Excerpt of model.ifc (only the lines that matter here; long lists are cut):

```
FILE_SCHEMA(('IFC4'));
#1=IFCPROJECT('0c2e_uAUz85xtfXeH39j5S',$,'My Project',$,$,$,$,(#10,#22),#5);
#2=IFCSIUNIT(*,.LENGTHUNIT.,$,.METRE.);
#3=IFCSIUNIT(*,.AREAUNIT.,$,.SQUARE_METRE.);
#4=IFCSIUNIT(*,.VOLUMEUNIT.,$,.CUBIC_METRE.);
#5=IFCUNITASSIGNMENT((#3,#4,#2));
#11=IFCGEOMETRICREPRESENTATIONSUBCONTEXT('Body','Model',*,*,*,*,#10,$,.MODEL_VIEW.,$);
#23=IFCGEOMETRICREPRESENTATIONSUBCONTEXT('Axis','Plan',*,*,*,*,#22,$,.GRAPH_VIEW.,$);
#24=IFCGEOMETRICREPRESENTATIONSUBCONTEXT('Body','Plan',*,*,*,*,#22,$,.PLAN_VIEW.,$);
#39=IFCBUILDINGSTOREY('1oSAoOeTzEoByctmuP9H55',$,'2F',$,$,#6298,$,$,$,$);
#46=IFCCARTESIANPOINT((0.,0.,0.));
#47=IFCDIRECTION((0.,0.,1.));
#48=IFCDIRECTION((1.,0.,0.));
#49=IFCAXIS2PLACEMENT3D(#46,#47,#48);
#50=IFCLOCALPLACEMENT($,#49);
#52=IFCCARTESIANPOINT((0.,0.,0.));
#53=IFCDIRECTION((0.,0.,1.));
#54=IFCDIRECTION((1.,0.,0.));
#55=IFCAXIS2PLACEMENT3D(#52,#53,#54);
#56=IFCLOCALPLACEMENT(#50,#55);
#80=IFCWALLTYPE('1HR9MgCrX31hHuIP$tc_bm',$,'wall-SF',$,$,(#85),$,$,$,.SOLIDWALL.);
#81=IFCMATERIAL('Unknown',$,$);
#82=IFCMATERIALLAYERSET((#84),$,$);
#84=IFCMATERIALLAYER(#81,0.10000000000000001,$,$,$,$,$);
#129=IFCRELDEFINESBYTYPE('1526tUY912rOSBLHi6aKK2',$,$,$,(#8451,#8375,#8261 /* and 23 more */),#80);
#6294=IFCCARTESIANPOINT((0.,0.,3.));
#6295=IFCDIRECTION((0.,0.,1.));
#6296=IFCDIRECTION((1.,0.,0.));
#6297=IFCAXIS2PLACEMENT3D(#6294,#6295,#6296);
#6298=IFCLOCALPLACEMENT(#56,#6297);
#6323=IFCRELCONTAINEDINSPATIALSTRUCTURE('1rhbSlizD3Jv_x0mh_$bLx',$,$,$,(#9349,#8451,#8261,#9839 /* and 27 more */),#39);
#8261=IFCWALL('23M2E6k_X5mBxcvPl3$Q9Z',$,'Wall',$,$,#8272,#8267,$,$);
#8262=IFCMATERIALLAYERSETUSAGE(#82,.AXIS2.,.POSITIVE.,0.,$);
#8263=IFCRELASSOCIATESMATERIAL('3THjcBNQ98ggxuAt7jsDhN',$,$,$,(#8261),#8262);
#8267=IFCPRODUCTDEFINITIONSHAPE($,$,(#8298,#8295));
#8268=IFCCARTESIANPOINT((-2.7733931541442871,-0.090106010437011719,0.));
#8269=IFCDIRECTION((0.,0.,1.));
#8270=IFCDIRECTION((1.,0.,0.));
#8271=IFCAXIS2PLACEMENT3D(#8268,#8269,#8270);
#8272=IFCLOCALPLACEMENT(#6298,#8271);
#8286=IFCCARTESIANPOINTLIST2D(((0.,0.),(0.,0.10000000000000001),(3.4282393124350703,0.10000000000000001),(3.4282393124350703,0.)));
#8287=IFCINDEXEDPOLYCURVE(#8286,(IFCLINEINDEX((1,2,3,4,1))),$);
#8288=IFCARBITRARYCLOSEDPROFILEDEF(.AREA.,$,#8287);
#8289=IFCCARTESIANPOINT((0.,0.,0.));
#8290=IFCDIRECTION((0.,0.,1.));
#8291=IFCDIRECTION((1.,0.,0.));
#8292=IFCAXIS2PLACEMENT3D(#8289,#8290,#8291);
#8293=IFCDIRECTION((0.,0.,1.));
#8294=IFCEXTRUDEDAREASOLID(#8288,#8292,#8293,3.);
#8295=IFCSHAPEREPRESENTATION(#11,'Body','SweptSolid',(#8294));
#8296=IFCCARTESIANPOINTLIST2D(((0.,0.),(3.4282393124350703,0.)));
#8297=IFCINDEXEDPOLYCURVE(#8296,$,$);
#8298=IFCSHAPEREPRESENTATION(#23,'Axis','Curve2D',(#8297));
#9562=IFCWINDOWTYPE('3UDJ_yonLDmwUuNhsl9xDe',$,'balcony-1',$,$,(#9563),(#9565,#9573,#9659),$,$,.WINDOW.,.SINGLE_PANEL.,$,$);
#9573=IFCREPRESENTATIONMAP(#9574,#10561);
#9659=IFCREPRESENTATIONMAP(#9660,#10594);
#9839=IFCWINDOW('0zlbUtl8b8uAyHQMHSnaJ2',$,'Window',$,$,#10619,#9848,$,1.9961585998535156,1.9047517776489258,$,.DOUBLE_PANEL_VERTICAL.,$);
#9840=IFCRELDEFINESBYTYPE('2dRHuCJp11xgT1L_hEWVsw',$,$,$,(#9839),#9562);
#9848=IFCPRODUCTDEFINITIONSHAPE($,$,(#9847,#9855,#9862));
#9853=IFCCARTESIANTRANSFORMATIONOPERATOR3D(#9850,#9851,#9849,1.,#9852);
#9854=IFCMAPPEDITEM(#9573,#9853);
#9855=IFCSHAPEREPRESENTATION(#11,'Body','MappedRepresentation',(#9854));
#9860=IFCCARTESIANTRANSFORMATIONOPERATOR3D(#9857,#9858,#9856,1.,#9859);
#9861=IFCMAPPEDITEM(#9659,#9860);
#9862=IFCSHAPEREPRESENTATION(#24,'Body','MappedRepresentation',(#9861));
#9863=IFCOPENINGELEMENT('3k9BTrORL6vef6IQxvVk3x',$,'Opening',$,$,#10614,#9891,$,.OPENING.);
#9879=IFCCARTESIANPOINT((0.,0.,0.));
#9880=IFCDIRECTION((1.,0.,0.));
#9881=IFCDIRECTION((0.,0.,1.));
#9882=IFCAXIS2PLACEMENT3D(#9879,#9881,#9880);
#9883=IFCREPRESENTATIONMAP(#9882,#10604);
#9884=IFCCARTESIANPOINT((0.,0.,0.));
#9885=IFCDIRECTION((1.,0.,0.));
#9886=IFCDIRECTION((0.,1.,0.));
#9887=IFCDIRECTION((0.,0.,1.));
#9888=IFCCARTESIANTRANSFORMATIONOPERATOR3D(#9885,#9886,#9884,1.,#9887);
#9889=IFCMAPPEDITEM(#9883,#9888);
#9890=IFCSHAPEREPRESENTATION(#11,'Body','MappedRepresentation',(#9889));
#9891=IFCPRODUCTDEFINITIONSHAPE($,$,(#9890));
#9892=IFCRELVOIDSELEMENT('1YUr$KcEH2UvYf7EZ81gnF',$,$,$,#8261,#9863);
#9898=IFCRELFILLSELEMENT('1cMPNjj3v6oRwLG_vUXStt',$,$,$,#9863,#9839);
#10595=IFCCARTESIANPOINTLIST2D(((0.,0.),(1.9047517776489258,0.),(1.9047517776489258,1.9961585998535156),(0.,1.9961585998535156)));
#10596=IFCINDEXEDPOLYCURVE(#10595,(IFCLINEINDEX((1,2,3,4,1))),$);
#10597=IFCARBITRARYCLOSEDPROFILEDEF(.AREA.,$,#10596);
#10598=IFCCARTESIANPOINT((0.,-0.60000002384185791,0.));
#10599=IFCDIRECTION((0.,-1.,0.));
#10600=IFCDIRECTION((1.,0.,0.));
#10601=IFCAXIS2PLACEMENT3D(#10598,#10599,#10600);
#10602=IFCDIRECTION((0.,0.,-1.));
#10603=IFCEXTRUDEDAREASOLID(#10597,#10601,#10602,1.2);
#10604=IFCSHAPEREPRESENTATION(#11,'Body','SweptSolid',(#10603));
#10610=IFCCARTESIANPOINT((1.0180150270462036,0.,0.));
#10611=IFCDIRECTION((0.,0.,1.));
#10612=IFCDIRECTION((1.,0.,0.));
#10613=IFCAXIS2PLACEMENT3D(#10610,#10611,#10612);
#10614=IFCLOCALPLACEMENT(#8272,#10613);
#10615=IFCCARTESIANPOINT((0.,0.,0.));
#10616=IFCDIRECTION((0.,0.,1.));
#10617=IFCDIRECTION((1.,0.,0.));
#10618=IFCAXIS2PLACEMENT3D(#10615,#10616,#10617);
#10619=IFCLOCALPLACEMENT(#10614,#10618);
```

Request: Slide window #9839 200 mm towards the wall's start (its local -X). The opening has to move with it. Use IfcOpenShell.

```python
import ifcopenshell
import ifcopenshell.api.geometry
import ifcopenshell.util.placement
import ifcopenshell.util.unit

model = ifcopenshell.open("model.ifc")
unit_scale = ifcopenshell.util.unit.calculate_unit_scale(model)

window = model.by_guid("0zlbUtl8b8uAyHQMHSnaJ2")
opening = window.FillsVoids[0].RelatingOpeningElement
wall = opening.VoidsElements[0].RelatingBuildingElement

wall_matrix = ifcopenshell.util.placement.get_local_placement(wall.ObjectPlacement)
shift = wall_matrix[:3, 0] * -0.2 / unit_scale
before = ifcopenshell.util.placement.get_local_placement(window.ObjectPlacement)[:3, 3].copy()

# The window is placed relative to its opening, so it follows when the opening moves.
matrix = ifcopenshell.util.placement.get_local_placement(opening.ObjectPlacement)
matrix[:3, 3] += shift
ifcopenshell.api.geometry.edit_object_placement(
    model, product=opening, matrix=matrix, is_si=False, should_transform_children=True
)

after = ifcopenshell.util.placement.get_local_placement(window.ObjectPlacement)[:3, 3]
print("window moved by", (after - before).round(3) + 0.0)

model.write("model_v2.ifc")
```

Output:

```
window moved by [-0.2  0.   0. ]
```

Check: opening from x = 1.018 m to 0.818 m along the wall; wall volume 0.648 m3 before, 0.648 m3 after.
